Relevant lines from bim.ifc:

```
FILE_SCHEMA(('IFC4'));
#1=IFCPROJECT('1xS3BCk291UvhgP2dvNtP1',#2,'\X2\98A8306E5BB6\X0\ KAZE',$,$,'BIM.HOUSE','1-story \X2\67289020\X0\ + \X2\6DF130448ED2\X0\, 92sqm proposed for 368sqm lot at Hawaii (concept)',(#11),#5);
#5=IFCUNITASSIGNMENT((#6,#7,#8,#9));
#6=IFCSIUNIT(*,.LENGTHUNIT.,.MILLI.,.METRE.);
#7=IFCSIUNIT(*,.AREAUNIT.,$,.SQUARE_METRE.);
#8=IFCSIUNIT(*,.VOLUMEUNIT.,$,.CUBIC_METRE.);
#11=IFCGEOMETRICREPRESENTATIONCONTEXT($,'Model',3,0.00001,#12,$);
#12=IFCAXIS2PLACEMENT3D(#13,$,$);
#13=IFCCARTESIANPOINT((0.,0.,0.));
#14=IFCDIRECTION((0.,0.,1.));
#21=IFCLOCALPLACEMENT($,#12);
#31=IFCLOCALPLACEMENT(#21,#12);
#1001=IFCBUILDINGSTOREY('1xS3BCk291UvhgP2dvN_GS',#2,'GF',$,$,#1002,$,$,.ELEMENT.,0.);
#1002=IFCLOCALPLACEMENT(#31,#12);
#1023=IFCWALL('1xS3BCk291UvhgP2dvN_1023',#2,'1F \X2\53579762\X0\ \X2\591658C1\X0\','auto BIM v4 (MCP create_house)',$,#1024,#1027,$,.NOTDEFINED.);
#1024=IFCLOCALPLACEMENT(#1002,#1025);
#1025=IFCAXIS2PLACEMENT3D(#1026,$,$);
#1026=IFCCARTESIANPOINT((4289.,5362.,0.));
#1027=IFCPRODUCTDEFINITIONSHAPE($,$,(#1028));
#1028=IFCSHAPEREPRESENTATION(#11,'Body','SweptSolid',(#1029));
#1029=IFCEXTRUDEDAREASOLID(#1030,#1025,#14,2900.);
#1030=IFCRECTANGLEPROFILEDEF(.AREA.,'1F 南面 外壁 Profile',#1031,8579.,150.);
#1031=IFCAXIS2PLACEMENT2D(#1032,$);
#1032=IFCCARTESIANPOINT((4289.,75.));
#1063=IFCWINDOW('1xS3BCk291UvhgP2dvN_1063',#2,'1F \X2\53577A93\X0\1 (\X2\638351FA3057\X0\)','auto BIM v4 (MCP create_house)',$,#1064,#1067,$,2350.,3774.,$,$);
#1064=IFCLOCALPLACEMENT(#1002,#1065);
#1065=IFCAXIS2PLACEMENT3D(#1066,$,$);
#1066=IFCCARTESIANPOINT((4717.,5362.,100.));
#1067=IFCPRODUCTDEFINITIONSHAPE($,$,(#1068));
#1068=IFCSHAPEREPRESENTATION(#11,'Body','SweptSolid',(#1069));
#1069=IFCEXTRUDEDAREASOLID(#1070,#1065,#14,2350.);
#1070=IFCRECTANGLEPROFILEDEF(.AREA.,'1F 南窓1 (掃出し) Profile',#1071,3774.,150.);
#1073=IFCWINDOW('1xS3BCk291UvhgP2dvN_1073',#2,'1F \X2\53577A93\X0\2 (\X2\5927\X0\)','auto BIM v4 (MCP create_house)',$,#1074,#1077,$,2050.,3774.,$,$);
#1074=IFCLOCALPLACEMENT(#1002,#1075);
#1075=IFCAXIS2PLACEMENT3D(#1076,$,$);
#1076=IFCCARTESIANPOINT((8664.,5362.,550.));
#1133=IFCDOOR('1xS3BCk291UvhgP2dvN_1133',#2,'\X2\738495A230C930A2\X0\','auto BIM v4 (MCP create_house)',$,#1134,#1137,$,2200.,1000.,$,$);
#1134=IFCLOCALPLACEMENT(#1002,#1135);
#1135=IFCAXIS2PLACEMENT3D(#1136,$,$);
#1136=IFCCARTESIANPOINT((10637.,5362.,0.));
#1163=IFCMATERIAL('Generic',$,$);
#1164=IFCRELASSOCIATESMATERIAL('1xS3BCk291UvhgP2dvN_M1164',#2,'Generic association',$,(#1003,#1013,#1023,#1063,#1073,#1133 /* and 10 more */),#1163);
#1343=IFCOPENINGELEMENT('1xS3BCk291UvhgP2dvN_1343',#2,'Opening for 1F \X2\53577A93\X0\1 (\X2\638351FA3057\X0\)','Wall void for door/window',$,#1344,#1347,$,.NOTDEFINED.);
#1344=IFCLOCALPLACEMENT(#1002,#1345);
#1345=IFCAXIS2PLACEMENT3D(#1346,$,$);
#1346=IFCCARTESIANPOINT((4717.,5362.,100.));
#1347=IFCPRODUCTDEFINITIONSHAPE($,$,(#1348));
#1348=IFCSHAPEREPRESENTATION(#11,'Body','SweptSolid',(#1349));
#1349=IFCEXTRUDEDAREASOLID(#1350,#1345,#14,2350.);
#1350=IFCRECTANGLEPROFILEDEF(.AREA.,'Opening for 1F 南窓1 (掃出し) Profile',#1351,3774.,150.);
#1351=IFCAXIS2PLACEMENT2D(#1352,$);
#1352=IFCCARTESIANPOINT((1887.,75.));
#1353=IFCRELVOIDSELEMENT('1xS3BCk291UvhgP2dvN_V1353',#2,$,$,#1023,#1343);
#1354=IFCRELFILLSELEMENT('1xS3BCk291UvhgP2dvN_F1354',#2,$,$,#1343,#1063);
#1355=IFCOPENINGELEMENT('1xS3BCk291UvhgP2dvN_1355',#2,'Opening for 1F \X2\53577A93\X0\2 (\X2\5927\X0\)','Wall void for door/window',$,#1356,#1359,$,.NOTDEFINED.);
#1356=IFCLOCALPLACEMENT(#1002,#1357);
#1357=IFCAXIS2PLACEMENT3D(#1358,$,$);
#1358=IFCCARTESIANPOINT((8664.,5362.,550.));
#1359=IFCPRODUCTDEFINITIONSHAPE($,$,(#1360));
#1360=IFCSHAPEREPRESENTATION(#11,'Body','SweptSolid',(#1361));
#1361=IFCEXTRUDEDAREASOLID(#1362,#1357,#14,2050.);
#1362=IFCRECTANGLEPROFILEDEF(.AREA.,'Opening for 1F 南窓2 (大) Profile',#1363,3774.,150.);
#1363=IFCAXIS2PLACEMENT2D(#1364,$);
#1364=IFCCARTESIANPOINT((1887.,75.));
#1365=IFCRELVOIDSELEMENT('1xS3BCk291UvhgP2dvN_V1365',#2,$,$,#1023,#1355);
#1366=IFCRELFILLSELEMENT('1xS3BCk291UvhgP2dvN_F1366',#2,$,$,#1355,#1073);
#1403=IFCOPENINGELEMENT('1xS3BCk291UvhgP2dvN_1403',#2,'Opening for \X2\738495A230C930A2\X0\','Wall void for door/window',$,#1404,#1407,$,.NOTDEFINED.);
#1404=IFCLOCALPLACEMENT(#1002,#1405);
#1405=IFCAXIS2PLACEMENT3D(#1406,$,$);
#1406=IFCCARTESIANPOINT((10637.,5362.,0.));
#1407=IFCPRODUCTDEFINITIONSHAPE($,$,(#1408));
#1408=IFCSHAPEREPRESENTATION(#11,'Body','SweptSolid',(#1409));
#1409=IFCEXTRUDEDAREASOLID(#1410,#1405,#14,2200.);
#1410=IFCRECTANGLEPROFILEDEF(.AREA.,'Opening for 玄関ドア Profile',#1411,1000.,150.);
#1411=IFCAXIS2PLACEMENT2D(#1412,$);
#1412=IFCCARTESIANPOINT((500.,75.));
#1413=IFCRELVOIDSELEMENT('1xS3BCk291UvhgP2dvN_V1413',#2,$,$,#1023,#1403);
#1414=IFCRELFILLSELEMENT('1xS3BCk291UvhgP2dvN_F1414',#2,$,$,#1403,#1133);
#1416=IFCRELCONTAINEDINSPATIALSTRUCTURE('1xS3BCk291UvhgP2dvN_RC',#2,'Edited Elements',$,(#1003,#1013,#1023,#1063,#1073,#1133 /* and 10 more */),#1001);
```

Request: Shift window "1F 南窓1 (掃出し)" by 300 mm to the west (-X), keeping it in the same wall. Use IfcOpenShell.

```python
import ifcopenshell
import ifcopenshell.api.geometry
import ifcopenshell.util.placement
import ifcopenshell.util.unit

model = ifcopenshell.open("bim.ifc")
unit_scale = ifcopenshell.util.unit.calculate_unit_scale(model)

window = model.by_guid("1xS3BCk291UvhgP2dvN_1063")
opening = window.FillsVoids[0].RelatingOpeningElement
wall = opening.VoidsElements[0].RelatingBuildingElement

wall_matrix = ifcopenshell.util.placement.get_local_placement(wall.ObjectPlacement)
shift = wall_matrix[:3, 0] * -0.3 / unit_scale
before = ifcopenshell.util.placement.get_local_placement(window.ObjectPlacement)[:3, 3].copy()

# The window is not placed relative to its opening, so move both.
for product in (opening, window):
    matrix = ifcopenshell.util.placement.get_local_placement(product.ObjectPlacement)
    matrix[:3, 3] += shift
    ifcopenshell.api.geometry.edit_object_placement(model, product=product, matrix=matrix, is_si=False)

after = ifcopenshell.util.placement.get_local_placement(window.ObjectPlacement)[:3, 3]
print("window moved by", (after - before).round(3) + 0.0)

model.write("bim-out.ifc")
```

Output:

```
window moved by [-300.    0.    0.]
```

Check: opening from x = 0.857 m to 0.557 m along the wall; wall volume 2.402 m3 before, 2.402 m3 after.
